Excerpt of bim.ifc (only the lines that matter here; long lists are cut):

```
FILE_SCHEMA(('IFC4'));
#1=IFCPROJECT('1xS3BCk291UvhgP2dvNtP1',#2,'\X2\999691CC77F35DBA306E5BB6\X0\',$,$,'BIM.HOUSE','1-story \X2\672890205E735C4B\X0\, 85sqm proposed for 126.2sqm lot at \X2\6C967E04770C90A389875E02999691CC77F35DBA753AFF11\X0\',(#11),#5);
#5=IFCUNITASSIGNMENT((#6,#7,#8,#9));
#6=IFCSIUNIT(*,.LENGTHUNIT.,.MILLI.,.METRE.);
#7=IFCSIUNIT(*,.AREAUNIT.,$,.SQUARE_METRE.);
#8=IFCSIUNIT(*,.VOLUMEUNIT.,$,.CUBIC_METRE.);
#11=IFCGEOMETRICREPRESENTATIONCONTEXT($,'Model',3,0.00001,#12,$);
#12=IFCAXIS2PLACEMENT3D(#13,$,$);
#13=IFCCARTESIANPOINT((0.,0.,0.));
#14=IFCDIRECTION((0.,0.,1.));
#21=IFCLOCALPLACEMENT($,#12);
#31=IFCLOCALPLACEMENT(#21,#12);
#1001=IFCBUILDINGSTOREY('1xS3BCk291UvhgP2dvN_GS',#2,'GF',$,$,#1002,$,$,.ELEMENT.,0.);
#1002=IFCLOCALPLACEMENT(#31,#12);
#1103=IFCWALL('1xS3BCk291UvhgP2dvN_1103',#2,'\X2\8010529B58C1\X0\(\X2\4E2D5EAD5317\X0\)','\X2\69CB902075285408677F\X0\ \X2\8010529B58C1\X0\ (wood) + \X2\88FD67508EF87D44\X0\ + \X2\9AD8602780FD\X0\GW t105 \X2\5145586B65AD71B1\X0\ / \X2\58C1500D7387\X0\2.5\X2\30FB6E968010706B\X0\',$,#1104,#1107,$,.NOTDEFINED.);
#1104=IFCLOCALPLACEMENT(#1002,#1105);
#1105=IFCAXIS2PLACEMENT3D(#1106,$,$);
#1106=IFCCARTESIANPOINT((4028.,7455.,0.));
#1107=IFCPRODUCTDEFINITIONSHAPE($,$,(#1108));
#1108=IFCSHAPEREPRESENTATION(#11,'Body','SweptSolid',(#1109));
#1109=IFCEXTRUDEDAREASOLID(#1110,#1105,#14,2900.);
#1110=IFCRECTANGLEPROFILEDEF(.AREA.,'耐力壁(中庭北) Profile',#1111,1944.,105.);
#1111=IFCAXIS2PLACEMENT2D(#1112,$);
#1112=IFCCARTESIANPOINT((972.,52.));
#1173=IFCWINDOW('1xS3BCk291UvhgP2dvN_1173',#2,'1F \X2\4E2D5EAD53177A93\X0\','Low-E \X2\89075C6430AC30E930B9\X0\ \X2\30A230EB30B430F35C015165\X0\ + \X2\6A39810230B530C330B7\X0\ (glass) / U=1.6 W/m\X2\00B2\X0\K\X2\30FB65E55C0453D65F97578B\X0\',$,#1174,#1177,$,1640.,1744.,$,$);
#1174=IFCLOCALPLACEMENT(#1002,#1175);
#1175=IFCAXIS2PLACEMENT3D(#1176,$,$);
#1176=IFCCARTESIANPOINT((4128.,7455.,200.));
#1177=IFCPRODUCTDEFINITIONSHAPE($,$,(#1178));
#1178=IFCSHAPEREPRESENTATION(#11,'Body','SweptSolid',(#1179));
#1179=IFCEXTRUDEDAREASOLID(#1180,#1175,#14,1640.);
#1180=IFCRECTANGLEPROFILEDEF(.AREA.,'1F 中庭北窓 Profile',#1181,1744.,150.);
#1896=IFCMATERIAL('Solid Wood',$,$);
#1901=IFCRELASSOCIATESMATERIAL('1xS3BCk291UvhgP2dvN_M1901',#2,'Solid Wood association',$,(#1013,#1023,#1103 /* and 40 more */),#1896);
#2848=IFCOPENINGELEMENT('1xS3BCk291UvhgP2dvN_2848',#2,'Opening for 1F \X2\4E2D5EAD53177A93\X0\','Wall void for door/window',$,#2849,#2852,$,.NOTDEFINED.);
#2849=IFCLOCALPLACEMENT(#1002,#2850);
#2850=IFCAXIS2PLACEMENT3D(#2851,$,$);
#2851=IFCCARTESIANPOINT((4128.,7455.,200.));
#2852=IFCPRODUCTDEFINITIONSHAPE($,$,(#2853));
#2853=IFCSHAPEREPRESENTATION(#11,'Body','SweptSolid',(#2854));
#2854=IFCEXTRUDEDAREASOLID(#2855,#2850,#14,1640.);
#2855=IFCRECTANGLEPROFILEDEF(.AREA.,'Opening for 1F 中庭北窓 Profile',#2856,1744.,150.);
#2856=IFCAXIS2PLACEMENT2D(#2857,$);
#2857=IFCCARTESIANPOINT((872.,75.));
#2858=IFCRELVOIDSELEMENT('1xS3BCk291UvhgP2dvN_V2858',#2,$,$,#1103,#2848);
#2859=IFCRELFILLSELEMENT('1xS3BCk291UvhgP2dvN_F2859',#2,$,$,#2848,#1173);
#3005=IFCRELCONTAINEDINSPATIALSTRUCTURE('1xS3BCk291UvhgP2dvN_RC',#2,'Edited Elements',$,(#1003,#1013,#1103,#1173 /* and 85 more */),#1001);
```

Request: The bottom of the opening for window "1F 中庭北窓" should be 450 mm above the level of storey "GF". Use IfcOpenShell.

```python
import numpy as np
import ifcopenshell
import ifcopenshell.api.geometry
import ifcopenshell.geom
import ifcopenshell.util.element
import ifcopenshell.util.placement
import ifcopenshell.util.shape
import ifcopenshell.util.unit

model = ifcopenshell.open("bim.ifc")
unit_scale = ifcopenshell.util.unit.calculate_unit_scale(model)

window = model.by_id(1173)
opening = window.FillsVoids[0].RelatingOpeningElement
storey = ifcopenshell.util.element.get_container(window, ifc_class="IfcBuildingStorey")
level = ifcopenshell.util.placement.get_local_placement(storey.ObjectPlacement)[2, 3]

# The opening's origin need not be at the sill, so measure its lowest point.
shape = ifcopenshell.geom.create_shape(ifcopenshell.geom.settings(), opening)
bottom = ifcopenshell.util.shape.get_shape_bottom_elevation(shape, shape.geometry) / unit_scale
dz = level + 0.45 / unit_scale - bottom

shift = np.array([0.0, 0.0, dz])
# The window is not placed relative to its opening, so move both.
for product in (opening, window):
    matrix = ifcopenshell.util.placement.get_local_placement(product.ObjectPlacement)
    matrix[:3, 3] += shift
    ifcopenshell.api.geometry.edit_object_placement(model, product=product, matrix=matrix, is_si=False)

print(f"moved by {dz * unit_scale:+.3f} m")

model.write("bim-out.ifc")
```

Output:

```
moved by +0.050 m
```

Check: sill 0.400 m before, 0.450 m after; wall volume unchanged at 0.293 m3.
